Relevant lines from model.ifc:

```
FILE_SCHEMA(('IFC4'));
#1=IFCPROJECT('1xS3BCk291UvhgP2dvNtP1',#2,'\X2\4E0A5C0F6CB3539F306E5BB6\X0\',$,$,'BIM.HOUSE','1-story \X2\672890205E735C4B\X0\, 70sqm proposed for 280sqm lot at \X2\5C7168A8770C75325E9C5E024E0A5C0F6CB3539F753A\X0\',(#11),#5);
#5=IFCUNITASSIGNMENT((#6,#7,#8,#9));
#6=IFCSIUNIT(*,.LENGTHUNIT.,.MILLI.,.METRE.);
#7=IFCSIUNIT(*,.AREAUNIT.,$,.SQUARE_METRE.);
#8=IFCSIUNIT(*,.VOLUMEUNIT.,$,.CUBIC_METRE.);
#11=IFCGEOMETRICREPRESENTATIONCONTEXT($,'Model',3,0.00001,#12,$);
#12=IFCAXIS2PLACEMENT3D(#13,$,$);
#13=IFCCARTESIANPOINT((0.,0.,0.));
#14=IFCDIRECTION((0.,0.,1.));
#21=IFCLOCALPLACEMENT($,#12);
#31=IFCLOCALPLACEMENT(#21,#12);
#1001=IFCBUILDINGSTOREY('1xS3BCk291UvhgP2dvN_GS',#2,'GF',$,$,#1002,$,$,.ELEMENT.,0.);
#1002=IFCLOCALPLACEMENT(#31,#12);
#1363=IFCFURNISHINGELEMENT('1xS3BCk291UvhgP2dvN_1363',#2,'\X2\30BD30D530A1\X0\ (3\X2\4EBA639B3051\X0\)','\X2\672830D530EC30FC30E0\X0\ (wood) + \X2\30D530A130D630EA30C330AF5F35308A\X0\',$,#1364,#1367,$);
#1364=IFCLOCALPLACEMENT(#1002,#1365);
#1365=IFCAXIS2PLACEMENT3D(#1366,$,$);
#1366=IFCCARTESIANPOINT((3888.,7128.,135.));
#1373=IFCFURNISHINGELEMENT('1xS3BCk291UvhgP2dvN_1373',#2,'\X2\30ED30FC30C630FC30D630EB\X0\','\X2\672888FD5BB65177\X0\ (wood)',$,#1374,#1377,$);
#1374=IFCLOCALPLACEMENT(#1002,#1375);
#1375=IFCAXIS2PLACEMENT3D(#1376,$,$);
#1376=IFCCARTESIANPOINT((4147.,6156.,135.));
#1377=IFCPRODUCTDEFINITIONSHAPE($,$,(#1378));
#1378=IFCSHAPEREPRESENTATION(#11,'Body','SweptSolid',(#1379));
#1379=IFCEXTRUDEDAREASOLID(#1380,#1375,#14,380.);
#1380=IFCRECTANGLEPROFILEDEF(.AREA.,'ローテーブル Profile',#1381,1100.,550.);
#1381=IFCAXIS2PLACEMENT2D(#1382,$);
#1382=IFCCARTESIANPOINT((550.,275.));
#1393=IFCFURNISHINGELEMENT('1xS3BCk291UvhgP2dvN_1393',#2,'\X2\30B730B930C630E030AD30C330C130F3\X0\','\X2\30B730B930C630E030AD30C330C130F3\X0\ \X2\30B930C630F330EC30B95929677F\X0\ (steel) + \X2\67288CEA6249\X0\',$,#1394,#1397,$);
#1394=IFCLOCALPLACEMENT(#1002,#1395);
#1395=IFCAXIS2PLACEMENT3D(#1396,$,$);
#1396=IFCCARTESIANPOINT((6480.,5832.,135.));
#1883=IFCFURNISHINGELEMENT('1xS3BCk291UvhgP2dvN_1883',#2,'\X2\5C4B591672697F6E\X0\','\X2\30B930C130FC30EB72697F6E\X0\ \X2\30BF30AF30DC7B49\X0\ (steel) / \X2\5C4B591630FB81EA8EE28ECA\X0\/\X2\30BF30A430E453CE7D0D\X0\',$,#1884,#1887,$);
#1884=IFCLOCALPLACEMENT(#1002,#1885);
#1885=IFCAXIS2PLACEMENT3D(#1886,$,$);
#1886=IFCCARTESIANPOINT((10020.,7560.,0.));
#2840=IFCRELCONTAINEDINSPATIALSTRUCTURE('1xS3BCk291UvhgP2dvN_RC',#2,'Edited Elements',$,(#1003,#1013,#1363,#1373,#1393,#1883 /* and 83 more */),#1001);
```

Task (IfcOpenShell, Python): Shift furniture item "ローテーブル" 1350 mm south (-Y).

```python
import ifcopenshell
import ifcopenshell.api.geometry
import ifcopenshell.util.placement
import ifcopenshell.util.unit

model = ifcopenshell.open("model.ifc")
unit_scale = ifcopenshell.util.unit.calculate_unit_scale(model)

item = model.by_guid("1xS3BCk291UvhgP2dvN_1373")
matrix = ifcopenshell.util.placement.get_local_placement(item.ObjectPlacement)
matrix[1, 3] -= 1.35 / unit_scale
ifcopenshell.api.geometry.edit_object_placement(model, product=item, matrix=matrix, is_si=False)

print(ifcopenshell.util.placement.get_local_placement(item.ObjectPlacement).round(3) + 0.0)

model.write("model_edited.ifc")
```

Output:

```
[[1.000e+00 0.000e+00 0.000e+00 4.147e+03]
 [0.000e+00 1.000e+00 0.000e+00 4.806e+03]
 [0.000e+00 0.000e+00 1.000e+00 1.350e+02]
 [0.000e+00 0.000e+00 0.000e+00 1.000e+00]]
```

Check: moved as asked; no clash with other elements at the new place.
